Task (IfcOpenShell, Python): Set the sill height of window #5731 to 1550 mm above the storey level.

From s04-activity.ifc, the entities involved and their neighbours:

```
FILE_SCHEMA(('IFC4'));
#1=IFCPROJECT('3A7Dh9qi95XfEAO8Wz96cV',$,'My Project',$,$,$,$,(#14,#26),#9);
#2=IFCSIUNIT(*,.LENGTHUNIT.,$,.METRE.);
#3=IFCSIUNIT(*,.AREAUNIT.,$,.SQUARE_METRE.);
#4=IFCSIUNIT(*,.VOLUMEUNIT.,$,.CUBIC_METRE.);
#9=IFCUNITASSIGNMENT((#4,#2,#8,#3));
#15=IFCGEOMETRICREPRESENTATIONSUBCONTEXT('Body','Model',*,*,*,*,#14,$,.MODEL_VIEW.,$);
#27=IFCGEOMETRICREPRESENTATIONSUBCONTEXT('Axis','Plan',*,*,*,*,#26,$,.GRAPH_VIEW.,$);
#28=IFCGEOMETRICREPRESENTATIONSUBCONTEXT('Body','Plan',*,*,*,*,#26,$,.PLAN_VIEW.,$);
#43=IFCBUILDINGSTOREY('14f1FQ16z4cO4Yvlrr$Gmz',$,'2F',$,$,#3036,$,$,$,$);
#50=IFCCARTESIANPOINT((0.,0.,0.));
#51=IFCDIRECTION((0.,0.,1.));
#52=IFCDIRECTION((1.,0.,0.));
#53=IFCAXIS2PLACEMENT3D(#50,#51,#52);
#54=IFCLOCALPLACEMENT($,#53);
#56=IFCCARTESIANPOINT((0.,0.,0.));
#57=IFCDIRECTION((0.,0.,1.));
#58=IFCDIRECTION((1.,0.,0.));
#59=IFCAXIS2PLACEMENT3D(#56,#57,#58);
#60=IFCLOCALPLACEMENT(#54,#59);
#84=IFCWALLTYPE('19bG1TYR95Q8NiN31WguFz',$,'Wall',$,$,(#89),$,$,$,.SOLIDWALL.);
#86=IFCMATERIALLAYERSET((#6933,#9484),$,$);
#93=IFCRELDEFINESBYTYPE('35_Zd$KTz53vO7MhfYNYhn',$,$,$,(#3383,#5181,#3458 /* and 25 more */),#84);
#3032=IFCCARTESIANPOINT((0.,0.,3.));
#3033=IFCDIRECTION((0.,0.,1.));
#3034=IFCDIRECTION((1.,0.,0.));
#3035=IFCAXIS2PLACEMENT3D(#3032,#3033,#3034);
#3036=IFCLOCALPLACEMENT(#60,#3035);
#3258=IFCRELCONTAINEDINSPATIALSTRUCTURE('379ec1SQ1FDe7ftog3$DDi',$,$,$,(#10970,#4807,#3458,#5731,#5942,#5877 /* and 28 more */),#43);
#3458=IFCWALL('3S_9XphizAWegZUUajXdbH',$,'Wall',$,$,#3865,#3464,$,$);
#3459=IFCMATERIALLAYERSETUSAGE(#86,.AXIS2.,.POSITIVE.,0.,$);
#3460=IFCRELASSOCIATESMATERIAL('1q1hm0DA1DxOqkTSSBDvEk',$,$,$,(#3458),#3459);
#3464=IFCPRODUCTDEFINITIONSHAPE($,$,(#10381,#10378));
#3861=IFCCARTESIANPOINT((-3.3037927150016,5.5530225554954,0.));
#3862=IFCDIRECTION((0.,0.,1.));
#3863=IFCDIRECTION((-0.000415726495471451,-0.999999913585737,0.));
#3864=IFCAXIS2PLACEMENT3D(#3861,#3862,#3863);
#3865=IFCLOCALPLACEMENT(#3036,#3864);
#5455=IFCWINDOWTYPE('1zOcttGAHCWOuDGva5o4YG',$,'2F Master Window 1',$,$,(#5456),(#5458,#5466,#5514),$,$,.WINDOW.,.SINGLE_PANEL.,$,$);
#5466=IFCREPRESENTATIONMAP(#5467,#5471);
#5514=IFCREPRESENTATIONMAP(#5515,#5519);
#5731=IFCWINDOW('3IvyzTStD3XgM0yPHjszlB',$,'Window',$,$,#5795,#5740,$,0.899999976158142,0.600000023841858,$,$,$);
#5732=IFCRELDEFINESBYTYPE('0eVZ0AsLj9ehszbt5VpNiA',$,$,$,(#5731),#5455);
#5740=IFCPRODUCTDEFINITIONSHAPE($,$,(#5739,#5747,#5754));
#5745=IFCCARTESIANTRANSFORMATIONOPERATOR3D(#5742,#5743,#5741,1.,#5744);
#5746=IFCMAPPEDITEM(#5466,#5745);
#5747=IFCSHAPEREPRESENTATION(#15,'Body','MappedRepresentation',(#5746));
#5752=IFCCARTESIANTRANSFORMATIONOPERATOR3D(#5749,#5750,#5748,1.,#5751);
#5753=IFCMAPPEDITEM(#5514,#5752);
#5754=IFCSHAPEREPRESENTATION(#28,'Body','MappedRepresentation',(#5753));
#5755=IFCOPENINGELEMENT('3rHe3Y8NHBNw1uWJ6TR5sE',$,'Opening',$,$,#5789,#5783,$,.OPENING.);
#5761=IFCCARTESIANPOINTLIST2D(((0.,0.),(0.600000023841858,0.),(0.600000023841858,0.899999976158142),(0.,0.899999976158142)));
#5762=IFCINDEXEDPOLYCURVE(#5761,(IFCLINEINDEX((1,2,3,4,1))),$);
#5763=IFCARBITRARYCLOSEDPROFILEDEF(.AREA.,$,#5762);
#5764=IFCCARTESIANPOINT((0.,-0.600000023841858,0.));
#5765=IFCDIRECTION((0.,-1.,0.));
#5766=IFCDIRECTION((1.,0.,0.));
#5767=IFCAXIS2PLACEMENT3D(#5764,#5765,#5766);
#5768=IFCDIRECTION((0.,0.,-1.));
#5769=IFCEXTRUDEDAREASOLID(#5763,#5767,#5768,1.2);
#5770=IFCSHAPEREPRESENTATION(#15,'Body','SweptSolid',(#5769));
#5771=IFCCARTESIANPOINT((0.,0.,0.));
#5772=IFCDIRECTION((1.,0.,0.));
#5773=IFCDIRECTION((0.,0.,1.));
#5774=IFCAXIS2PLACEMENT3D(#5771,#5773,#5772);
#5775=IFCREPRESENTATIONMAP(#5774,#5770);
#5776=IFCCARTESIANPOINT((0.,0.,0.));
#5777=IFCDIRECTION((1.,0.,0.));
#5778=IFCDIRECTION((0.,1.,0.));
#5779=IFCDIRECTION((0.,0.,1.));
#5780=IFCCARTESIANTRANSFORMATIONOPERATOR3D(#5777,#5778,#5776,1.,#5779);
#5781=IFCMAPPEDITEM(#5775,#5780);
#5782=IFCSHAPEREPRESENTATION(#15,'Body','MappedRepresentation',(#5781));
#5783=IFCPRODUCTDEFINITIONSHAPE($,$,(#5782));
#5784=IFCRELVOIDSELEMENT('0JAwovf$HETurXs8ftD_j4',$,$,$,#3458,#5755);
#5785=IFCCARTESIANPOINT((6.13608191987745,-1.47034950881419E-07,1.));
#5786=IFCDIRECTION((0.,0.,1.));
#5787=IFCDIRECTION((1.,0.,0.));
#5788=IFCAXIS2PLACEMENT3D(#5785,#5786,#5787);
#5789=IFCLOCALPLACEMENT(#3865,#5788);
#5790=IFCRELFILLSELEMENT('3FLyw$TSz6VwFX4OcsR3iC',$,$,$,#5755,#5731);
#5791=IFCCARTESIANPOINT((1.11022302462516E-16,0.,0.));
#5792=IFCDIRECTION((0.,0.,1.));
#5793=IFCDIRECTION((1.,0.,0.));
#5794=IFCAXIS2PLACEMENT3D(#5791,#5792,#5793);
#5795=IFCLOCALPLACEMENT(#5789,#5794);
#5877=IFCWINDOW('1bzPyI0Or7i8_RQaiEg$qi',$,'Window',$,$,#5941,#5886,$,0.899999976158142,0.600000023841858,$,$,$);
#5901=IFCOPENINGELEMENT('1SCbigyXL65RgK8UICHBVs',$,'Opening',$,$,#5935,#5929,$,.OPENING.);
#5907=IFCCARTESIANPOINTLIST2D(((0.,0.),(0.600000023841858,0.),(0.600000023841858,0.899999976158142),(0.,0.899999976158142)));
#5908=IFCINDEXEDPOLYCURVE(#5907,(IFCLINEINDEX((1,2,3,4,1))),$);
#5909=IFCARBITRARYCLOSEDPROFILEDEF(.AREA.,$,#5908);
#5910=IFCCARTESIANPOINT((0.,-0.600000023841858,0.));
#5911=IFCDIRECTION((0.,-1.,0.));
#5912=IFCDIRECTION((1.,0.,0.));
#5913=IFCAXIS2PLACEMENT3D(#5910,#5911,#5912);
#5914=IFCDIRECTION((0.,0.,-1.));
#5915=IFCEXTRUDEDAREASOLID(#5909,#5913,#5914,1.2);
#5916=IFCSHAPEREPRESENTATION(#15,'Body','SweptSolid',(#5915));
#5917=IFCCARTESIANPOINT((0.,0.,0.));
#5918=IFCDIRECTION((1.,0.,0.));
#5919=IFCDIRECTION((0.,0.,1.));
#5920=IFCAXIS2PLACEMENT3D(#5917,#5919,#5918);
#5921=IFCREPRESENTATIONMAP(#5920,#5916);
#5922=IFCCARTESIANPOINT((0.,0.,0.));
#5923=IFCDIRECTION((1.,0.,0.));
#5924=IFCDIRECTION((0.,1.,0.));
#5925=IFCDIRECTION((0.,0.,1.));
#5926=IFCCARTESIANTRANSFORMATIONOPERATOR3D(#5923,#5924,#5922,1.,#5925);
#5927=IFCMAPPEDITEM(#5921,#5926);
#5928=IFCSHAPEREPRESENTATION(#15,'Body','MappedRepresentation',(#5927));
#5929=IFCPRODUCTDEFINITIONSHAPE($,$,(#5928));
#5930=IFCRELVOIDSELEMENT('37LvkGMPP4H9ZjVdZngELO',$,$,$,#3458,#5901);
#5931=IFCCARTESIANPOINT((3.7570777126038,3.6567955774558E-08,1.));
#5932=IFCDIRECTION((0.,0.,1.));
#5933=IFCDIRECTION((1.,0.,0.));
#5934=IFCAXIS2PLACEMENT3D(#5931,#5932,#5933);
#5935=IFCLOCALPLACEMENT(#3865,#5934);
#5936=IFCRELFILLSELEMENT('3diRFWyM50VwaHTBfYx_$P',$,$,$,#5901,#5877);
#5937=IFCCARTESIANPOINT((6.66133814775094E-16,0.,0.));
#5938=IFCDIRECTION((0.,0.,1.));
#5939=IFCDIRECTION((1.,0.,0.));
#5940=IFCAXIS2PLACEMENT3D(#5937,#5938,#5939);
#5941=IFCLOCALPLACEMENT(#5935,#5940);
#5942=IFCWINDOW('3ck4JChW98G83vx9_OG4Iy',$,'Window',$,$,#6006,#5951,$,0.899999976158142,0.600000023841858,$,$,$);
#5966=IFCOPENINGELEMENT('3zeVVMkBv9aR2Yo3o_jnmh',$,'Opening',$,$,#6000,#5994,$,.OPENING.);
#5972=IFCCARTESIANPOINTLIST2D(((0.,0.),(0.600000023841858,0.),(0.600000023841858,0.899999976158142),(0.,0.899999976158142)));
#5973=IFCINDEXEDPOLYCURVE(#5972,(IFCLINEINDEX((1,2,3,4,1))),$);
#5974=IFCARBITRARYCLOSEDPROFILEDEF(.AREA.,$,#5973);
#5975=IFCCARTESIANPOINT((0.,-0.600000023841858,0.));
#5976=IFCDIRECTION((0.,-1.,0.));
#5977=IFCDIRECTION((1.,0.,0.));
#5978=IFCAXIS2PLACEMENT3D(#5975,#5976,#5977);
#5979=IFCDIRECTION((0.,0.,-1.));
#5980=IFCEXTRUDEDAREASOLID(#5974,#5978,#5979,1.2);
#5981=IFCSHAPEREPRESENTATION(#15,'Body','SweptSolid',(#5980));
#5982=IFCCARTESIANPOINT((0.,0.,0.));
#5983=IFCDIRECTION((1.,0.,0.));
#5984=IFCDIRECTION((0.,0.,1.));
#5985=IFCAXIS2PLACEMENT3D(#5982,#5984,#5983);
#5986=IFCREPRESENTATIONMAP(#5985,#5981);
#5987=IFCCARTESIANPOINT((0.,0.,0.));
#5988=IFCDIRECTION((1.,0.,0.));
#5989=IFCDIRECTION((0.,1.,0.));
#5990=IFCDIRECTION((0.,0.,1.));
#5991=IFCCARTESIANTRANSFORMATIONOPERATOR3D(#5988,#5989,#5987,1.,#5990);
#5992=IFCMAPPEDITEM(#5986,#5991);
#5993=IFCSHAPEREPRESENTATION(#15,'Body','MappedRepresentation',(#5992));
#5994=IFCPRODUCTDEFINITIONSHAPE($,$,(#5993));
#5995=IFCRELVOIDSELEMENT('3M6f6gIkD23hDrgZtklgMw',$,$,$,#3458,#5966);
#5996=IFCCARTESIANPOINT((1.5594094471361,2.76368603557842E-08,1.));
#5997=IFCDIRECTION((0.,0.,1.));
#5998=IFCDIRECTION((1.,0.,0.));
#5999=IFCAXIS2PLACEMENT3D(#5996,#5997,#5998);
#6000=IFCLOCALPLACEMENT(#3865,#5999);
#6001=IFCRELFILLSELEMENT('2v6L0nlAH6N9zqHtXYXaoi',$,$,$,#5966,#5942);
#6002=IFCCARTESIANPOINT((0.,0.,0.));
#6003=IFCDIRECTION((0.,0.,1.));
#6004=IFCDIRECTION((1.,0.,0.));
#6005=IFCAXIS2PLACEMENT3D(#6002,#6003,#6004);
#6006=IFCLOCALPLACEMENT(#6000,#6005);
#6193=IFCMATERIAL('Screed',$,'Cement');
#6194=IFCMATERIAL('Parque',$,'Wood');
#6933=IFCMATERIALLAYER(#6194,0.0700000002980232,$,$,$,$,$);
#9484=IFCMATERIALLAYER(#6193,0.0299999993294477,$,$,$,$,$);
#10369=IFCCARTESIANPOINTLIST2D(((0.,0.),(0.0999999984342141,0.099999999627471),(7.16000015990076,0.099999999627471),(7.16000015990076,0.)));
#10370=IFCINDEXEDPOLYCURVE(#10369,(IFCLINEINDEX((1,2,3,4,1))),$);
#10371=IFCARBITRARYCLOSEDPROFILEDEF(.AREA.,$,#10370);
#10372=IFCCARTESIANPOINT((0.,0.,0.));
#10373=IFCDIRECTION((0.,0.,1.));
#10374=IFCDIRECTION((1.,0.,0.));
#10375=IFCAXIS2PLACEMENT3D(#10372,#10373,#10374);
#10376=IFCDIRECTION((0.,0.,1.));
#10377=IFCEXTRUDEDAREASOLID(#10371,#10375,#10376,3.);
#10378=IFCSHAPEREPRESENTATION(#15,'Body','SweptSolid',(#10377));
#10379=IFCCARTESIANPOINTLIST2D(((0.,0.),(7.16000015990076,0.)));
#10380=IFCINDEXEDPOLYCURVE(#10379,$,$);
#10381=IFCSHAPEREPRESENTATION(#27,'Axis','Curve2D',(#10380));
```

```python
import numpy as np
import ifcopenshell
import ifcopenshell.api.geometry
import ifcopenshell.geom
import ifcopenshell.util.element
import ifcopenshell.util.placement
import ifcopenshell.util.shape
import ifcopenshell.util.unit

model = ifcopenshell.open("s04-activity.ifc")
unit_scale = ifcopenshell.util.unit.calculate_unit_scale(model)

window = model.by_guid("3IvyzTStD3XgM0yPHjszlB")
opening = window.FillsVoids[0].RelatingOpeningElement
storey = ifcopenshell.util.element.get_container(window, ifc_class="IfcBuildingStorey")
level = ifcopenshell.util.placement.get_local_placement(storey.ObjectPlacement)[2, 3]

# The opening's origin need not be at the sill, so measure its lowest point.
shape = ifcopenshell.geom.create_shape(ifcopenshell.geom.settings(), opening)
bottom = ifcopenshell.util.shape.get_shape_bottom_elevation(shape, shape.geometry) / unit_scale
dz = level + 1.55 / unit_scale - bottom

shift = np.array([0.0, 0.0, dz])
# The window is placed relative to its opening, so it follows when the opening moves.
matrix = ifcopenshell.util.placement.get_local_placement(opening.ObjectPlacement)
matrix[:3, 3] += shift
ifcopenshell.api.geometry.edit_object_placement(
    model, product=opening, matrix=matrix, is_si=False, should_transform_children=True
)

print(f"moved by {dz * unit_scale:+.3f} m")

model.write("s04-activity-out.ifc")
```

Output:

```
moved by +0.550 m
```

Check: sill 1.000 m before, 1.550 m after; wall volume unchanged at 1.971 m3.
